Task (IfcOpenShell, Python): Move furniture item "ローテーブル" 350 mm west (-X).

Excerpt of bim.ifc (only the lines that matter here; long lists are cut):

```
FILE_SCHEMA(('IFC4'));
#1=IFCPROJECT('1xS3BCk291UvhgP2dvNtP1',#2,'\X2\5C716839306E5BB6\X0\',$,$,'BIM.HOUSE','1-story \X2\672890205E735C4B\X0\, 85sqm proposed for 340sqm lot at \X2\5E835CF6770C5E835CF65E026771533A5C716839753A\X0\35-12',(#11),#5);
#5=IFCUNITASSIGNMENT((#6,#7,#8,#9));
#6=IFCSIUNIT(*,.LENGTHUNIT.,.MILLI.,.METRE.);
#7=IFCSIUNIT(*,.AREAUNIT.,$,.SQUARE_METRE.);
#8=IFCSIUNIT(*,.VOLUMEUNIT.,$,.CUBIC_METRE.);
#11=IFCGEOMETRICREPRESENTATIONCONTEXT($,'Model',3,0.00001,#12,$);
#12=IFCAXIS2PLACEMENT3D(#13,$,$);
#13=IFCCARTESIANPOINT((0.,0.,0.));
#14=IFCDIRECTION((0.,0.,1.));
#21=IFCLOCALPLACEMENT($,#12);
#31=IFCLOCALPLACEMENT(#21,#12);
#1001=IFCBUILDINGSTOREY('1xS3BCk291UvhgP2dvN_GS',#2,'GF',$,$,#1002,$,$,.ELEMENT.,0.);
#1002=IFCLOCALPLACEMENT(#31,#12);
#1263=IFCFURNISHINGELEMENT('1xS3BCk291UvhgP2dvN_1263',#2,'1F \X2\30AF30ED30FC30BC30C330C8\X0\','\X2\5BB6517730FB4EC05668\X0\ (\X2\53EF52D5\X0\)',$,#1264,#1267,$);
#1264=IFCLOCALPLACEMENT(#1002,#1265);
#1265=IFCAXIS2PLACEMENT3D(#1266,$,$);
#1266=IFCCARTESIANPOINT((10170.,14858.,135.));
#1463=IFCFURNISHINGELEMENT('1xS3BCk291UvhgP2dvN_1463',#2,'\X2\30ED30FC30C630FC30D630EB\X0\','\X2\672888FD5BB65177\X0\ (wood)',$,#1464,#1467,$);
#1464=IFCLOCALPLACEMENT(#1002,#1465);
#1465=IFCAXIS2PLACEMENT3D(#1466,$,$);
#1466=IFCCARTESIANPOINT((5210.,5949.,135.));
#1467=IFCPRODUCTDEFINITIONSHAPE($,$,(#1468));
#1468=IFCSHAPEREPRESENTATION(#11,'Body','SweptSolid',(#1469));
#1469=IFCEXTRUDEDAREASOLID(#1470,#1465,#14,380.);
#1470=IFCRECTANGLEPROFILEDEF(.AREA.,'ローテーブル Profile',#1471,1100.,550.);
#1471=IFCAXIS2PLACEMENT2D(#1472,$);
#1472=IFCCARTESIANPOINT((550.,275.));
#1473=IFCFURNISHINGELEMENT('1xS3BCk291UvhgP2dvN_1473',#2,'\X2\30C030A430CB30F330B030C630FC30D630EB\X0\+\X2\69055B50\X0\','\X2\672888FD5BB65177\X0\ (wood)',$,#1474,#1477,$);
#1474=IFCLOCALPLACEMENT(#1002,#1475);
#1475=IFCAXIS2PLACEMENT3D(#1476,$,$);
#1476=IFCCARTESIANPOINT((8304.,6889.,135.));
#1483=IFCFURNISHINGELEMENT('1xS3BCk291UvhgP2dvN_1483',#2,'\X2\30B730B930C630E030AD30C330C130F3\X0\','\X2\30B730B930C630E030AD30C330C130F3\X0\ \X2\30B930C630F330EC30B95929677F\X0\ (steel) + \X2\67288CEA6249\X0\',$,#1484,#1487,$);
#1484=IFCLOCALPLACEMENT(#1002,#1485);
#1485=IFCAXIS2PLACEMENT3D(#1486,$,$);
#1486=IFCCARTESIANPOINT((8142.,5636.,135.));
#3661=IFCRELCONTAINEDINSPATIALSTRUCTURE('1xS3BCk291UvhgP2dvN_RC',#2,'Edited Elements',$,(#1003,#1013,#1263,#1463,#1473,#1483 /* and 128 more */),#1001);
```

```python
import ifcopenshell
import ifcopenshell.api.geometry
import ifcopenshell.util.placement
import ifcopenshell.util.unit

model = ifcopenshell.open("bim.ifc")
unit_scale = ifcopenshell.util.unit.calculate_unit_scale(model)

item = model.by_id(1463)
matrix = ifcopenshell.util.placement.get_local_placement(item.ObjectPlacement)
matrix[0, 3] -= 0.35 / unit_scale
ifcopenshell.api.geometry.edit_object_placement(model, product=item, matrix=matrix, is_si=False)

print(ifcopenshell.util.placement.get_local_placement(item.ObjectPlacement).round(3) + 0.0)

model.write("bim_edited.ifc")
```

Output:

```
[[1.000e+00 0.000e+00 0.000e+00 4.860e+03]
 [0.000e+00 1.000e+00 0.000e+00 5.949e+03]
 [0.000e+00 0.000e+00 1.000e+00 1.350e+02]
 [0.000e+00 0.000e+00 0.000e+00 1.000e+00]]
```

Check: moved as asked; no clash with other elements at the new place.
